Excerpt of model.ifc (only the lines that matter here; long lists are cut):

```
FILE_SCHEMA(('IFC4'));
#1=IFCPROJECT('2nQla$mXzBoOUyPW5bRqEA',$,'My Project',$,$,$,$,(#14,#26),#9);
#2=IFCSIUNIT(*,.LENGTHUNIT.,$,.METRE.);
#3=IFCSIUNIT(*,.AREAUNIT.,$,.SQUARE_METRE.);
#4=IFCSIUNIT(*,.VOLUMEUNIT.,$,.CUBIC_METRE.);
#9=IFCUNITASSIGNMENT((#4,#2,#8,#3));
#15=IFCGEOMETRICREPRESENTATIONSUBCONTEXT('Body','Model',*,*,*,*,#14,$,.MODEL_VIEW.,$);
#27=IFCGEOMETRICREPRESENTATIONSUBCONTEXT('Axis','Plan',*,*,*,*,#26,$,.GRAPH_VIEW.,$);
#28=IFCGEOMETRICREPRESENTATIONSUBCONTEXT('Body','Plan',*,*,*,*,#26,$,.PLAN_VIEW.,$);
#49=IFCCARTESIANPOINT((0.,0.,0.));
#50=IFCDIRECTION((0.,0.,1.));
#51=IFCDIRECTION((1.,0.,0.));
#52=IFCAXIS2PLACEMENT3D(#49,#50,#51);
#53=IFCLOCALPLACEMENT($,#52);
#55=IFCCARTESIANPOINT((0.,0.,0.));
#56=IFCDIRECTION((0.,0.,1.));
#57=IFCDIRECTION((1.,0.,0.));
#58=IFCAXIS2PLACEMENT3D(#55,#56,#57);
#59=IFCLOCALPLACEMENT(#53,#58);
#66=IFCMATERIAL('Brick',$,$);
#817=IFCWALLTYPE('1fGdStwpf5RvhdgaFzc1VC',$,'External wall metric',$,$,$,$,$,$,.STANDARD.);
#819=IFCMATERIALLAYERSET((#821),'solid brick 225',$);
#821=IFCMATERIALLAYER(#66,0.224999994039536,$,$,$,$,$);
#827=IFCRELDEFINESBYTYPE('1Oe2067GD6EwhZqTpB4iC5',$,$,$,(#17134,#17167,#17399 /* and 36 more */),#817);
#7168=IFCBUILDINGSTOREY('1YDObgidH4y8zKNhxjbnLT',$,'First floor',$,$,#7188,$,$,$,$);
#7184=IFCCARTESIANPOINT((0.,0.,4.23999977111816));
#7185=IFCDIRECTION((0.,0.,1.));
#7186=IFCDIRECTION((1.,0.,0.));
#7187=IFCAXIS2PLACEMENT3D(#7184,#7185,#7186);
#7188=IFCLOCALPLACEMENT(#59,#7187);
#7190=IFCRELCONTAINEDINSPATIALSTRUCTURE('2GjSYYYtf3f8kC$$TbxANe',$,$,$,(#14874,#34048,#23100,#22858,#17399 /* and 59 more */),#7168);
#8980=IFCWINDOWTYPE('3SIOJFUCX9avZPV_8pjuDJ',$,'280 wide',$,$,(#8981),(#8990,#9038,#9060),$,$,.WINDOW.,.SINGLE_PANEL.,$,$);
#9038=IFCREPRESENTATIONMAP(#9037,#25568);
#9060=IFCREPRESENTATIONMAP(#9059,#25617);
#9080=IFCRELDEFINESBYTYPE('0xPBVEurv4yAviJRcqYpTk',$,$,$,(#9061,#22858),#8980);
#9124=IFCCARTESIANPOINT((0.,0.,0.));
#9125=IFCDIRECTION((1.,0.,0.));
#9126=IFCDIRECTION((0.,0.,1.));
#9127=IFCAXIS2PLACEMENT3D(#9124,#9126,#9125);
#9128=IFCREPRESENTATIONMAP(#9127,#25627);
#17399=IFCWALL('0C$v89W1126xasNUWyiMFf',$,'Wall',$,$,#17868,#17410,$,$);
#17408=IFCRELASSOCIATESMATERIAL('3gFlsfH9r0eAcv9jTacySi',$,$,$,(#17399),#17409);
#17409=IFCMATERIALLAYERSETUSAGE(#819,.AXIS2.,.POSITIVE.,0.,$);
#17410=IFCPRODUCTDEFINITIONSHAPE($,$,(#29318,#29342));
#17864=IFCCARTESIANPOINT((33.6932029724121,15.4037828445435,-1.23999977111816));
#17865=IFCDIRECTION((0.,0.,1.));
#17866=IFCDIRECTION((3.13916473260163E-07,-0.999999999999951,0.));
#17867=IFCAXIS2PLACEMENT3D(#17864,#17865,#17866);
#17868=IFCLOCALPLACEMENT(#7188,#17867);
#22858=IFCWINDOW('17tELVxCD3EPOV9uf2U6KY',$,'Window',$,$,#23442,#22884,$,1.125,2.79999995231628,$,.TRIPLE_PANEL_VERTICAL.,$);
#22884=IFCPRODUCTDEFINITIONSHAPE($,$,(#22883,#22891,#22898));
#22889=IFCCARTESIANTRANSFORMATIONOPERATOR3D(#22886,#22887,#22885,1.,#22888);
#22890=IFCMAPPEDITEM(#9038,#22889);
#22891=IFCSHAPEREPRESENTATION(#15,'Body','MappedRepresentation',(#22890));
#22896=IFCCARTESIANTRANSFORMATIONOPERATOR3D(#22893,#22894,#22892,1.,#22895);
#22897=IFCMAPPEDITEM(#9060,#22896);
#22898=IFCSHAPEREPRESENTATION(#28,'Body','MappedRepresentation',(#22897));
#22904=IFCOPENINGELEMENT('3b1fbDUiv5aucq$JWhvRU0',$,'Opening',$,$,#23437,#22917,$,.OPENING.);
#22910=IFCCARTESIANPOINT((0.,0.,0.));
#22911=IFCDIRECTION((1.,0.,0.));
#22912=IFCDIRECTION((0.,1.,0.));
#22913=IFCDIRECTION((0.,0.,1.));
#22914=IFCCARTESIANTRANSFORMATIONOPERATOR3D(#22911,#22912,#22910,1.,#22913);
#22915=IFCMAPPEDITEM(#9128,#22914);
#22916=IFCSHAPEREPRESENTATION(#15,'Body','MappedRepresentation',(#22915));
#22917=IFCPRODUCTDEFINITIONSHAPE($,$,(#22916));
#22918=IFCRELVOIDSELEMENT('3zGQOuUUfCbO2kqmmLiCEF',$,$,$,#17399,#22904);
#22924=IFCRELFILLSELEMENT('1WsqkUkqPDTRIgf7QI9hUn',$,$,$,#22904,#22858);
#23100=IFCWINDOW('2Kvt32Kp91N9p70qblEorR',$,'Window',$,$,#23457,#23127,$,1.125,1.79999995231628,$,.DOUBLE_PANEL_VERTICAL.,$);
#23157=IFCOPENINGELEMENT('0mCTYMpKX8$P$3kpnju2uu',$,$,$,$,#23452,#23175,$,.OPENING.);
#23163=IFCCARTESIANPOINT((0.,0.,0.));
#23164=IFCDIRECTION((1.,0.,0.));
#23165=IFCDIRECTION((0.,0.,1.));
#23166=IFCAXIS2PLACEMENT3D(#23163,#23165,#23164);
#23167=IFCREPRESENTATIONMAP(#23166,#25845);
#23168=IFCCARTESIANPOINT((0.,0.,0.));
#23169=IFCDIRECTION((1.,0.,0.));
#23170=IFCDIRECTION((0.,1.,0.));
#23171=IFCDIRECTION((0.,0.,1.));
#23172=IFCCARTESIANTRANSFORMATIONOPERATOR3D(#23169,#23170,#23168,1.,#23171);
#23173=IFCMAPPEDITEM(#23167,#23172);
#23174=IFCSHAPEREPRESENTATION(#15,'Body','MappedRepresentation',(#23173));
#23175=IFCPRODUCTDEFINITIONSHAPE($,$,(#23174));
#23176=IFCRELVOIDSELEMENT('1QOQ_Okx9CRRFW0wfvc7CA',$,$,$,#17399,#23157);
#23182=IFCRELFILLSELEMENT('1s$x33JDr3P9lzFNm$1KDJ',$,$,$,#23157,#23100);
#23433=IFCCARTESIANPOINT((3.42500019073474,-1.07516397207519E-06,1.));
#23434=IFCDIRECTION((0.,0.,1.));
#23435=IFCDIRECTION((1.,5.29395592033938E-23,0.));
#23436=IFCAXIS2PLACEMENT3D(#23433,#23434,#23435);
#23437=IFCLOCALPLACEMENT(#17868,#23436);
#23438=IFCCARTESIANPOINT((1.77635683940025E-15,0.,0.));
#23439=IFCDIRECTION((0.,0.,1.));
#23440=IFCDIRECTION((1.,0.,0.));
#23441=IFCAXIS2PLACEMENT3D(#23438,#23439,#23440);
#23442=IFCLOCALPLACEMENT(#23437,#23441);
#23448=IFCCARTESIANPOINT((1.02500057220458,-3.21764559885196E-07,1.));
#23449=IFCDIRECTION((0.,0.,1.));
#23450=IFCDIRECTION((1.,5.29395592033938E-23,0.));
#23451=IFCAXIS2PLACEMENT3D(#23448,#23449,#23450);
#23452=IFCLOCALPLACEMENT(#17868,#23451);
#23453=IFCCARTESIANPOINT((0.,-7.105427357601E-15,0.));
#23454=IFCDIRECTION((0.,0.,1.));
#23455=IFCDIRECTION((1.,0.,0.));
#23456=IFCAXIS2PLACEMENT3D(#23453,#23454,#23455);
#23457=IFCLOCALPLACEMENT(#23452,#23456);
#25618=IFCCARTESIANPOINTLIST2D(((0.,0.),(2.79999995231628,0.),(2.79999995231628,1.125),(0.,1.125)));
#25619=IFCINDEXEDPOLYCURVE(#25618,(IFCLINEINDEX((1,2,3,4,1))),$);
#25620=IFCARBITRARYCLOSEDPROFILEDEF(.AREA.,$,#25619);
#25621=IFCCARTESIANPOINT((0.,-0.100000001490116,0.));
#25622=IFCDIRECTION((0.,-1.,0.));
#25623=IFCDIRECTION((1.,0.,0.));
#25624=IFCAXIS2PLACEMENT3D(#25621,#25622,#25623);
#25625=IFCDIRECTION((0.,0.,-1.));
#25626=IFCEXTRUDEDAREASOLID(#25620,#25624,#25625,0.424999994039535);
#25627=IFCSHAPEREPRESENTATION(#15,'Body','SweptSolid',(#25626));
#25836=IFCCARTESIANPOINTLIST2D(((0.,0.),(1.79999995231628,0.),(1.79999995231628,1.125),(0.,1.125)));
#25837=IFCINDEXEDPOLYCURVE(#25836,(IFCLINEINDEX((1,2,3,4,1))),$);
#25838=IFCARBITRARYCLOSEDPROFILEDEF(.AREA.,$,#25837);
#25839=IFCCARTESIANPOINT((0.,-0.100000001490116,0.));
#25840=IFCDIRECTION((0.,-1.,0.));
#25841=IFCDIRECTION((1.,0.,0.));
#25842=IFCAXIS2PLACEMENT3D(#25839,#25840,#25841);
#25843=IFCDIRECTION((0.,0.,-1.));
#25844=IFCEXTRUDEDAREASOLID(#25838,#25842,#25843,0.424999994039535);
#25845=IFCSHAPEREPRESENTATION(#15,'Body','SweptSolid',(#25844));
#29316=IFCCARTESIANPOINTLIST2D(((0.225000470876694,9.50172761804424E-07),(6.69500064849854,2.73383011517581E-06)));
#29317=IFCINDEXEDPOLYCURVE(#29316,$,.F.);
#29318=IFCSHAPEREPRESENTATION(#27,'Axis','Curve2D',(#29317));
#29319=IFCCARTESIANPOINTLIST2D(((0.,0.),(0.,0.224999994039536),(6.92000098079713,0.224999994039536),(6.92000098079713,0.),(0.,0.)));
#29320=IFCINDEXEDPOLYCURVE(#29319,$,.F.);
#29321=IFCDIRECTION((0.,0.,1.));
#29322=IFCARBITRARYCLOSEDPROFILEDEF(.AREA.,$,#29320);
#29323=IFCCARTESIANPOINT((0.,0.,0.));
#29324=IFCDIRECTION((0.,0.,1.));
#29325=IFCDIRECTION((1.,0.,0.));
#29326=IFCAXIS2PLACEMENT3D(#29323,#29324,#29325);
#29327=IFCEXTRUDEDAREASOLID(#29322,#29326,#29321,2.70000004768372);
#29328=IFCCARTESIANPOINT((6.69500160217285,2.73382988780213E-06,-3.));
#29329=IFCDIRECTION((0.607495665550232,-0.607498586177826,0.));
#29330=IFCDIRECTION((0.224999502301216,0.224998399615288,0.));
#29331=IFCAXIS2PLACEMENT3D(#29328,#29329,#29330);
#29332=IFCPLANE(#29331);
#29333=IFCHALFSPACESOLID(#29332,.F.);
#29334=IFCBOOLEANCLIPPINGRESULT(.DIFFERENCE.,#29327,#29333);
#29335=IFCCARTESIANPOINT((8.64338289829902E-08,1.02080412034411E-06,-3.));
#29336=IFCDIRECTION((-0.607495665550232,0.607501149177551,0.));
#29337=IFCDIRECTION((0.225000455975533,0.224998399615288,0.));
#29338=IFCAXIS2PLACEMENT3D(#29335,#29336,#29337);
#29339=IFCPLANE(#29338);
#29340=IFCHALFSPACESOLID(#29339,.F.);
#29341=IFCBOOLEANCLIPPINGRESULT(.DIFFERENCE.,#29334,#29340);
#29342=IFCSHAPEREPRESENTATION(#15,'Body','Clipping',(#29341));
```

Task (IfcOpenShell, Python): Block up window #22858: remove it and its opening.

```python
import ifcopenshell
import ifcopenshell.api.feature
import ifcopenshell.api.root
import ifcopenshell.geom
import ifcopenshell.util.shape

model = ifcopenshell.open("model.ifc")
settings = ifcopenshell.geom.settings()


def volume(element):
    """Net volume in cubic metres, openings subtracted."""
    shape = ifcopenshell.geom.create_shape(settings, element)
    return ifcopenshell.util.shape.get_volume(shape.geometry)


window = model.by_guid("17tELVxCD3EPOV9uf2U6KY")
opening = window.FillsVoids[0].RelatingOpeningElement
wall = opening.VoidsElements[0].RelatingBuildingElement
before = volume(wall)

ifcopenshell.api.root.remove_product(model, product=window)
ifcopenshell.api.feature.remove_feature(model, feature=opening)

after = volume(wall)

print(f"wall volume {before:.3f} -> {after:.3f} m3")

model.write("model_edited.ifc")
```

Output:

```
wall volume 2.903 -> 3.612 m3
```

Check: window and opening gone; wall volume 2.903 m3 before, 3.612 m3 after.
